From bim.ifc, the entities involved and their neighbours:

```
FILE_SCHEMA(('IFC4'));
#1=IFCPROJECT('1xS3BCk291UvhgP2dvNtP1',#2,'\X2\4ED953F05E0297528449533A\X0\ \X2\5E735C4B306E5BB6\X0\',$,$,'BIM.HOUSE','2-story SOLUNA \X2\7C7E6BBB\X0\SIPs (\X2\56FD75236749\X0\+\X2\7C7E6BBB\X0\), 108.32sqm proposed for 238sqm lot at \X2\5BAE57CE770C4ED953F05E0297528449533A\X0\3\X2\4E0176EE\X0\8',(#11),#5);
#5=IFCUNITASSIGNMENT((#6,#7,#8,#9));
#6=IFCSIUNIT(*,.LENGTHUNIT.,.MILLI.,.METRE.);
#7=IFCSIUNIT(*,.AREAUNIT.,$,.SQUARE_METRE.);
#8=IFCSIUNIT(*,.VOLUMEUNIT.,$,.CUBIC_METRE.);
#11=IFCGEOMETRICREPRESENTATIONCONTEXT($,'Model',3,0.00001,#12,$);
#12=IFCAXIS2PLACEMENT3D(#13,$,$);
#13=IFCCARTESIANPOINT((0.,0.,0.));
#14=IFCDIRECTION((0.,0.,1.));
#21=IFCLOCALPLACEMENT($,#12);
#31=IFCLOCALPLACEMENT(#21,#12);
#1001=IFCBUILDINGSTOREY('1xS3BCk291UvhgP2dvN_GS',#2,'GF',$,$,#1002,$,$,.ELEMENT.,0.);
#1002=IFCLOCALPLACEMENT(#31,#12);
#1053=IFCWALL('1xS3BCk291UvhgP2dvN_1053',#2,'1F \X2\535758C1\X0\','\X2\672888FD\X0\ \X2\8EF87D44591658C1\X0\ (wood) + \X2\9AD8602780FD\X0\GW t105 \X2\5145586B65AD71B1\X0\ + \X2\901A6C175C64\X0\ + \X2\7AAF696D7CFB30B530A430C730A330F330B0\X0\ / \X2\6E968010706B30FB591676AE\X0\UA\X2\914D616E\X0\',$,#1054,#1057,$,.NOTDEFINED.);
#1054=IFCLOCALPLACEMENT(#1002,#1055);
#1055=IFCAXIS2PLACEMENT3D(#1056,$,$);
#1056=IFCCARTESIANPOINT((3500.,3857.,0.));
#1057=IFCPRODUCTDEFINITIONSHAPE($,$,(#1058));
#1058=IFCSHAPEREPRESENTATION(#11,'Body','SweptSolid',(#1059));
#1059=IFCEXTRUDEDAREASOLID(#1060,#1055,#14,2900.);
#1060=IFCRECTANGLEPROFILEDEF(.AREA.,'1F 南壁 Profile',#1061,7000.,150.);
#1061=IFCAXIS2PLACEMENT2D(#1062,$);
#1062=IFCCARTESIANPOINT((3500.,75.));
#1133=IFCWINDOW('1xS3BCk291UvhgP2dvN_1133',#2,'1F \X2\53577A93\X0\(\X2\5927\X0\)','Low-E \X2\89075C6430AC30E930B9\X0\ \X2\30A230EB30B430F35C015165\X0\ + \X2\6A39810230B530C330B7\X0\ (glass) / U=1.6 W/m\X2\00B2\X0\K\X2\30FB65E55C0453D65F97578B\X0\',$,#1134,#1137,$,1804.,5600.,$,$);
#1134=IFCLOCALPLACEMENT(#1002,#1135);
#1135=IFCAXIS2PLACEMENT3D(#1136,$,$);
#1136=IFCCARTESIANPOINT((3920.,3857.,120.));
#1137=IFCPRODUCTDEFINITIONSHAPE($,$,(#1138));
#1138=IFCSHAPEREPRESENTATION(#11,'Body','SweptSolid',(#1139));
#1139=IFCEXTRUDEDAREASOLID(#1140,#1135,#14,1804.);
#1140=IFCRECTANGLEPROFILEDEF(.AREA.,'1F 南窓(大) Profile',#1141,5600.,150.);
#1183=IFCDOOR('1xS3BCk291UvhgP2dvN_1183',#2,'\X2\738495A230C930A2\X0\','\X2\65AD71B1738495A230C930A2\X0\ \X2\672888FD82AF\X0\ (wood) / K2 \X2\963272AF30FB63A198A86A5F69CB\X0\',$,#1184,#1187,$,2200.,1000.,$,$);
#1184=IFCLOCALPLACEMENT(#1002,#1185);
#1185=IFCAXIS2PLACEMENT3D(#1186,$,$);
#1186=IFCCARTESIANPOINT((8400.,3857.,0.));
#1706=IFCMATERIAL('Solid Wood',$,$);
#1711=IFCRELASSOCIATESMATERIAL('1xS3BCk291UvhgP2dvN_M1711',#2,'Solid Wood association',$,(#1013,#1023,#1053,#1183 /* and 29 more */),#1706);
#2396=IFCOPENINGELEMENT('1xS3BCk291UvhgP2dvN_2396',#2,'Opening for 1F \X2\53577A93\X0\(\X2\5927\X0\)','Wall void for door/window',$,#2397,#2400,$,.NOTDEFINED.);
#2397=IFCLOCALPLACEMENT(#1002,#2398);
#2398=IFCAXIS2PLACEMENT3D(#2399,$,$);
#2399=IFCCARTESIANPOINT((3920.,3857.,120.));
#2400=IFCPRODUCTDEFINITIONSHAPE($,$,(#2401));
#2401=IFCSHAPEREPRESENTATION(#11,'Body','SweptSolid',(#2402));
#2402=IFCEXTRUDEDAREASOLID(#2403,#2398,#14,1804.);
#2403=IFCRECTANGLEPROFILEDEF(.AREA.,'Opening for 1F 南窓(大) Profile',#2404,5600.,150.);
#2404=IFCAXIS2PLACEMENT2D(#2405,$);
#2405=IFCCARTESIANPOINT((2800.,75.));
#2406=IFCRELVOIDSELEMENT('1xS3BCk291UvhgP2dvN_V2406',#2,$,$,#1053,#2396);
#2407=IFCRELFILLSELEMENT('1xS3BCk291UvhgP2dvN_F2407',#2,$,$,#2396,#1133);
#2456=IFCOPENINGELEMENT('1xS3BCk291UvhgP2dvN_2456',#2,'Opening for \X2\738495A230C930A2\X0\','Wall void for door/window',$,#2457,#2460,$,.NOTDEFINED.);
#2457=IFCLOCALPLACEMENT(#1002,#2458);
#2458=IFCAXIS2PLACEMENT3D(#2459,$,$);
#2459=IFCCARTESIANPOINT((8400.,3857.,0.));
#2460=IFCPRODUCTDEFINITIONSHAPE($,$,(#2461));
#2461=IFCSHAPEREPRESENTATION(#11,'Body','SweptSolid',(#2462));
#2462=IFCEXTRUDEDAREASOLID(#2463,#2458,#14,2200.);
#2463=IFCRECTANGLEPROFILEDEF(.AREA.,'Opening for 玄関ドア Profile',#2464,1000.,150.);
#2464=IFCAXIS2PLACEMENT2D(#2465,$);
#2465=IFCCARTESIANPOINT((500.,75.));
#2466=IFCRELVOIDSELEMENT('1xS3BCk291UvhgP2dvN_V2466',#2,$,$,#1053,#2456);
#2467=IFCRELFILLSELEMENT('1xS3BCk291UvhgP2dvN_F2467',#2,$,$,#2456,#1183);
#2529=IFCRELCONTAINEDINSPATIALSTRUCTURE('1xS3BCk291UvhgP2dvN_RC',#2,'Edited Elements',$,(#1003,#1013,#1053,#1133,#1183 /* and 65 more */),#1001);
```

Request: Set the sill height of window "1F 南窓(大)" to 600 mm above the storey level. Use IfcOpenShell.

```python
import numpy as np
import ifcopenshell
import ifcopenshell.api.geometry
import ifcopenshell.geom
import ifcopenshell.util.element
import ifcopenshell.util.placement
import ifcopenshell.util.shape
import ifcopenshell.util.unit

model = ifcopenshell.open("bim.ifc")
unit_scale = ifcopenshell.util.unit.calculate_unit_scale(model)

window = model.by_guid("1xS3BCk291UvhgP2dvN_1133")
opening = window.FillsVoids[0].RelatingOpeningElement
storey = ifcopenshell.util.element.get_container(window, ifc_class="IfcBuildingStorey")
level = ifcopenshell.util.placement.get_local_placement(storey.ObjectPlacement)[2, 3]

# The opening's origin need not be at the sill, so measure its lowest point.
shape = ifcopenshell.geom.create_shape(ifcopenshell.geom.settings(), opening)
bottom = ifcopenshell.util.shape.get_shape_bottom_elevation(shape, shape.geometry) / unit_scale
dz = level + 0.6 / unit_scale - bottom

shift = np.array([0.0, 0.0, dz])
# The window is not placed relative to its opening, so move both.
for product in (opening, window):
    matrix = ifcopenshell.util.placement.get_local_placement(product.ObjectPlacement)
    matrix[:3, 3] += shift
    ifcopenshell.api.geometry.edit_object_placement(model, product=product, matrix=matrix, is_si=False)

print(f"moved by {dz * unit_scale:+.3f} m")

model.write("bim-out.ifc")
```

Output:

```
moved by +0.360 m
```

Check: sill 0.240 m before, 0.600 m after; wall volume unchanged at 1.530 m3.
